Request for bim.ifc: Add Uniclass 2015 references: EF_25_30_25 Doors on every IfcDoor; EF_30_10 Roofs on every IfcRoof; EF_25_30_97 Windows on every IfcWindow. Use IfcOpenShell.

First a look at what the model holds.

```python
import ifcopenshell

model = ifcopenshell.open("bim.ifc")
print(model.schema)
print("classifications:", [c.Name for c in model.by_type("IfcClassification")])
for ifc_class in ("IfcDoor", "IfcRoof", "IfcStair", "IfcWall", "IfcWindow"):
    print(ifc_class, len(model.by_type(ifc_class)))
```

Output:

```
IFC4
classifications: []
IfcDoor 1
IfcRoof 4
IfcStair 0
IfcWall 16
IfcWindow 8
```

```python
import ifcopenshell
import ifcopenshell.api.classification

model = ifcopenshell.open("bim.ifc")

system = ifcopenshell.api.classification.add_classification(model, classification="Uniclass 2015")

codes = {
    "IfcDoor": ("EF_25_30_25", "Doors"),
    "IfcRoof": ("EF_30_10", "Roofs"),
    "IfcWindow": ("EF_25_30_97", "Windows"),
}
for ifc_class, (code, name) in codes.items():
    products = model.by_type(ifc_class)
    ifcopenshell.api.classification.add_reference(
        model, products=products, classification=system, identification=code, name=name
    )
    print(code, len(products))

model.write("bim-out.ifc")
```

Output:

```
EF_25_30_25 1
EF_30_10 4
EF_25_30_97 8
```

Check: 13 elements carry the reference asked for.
